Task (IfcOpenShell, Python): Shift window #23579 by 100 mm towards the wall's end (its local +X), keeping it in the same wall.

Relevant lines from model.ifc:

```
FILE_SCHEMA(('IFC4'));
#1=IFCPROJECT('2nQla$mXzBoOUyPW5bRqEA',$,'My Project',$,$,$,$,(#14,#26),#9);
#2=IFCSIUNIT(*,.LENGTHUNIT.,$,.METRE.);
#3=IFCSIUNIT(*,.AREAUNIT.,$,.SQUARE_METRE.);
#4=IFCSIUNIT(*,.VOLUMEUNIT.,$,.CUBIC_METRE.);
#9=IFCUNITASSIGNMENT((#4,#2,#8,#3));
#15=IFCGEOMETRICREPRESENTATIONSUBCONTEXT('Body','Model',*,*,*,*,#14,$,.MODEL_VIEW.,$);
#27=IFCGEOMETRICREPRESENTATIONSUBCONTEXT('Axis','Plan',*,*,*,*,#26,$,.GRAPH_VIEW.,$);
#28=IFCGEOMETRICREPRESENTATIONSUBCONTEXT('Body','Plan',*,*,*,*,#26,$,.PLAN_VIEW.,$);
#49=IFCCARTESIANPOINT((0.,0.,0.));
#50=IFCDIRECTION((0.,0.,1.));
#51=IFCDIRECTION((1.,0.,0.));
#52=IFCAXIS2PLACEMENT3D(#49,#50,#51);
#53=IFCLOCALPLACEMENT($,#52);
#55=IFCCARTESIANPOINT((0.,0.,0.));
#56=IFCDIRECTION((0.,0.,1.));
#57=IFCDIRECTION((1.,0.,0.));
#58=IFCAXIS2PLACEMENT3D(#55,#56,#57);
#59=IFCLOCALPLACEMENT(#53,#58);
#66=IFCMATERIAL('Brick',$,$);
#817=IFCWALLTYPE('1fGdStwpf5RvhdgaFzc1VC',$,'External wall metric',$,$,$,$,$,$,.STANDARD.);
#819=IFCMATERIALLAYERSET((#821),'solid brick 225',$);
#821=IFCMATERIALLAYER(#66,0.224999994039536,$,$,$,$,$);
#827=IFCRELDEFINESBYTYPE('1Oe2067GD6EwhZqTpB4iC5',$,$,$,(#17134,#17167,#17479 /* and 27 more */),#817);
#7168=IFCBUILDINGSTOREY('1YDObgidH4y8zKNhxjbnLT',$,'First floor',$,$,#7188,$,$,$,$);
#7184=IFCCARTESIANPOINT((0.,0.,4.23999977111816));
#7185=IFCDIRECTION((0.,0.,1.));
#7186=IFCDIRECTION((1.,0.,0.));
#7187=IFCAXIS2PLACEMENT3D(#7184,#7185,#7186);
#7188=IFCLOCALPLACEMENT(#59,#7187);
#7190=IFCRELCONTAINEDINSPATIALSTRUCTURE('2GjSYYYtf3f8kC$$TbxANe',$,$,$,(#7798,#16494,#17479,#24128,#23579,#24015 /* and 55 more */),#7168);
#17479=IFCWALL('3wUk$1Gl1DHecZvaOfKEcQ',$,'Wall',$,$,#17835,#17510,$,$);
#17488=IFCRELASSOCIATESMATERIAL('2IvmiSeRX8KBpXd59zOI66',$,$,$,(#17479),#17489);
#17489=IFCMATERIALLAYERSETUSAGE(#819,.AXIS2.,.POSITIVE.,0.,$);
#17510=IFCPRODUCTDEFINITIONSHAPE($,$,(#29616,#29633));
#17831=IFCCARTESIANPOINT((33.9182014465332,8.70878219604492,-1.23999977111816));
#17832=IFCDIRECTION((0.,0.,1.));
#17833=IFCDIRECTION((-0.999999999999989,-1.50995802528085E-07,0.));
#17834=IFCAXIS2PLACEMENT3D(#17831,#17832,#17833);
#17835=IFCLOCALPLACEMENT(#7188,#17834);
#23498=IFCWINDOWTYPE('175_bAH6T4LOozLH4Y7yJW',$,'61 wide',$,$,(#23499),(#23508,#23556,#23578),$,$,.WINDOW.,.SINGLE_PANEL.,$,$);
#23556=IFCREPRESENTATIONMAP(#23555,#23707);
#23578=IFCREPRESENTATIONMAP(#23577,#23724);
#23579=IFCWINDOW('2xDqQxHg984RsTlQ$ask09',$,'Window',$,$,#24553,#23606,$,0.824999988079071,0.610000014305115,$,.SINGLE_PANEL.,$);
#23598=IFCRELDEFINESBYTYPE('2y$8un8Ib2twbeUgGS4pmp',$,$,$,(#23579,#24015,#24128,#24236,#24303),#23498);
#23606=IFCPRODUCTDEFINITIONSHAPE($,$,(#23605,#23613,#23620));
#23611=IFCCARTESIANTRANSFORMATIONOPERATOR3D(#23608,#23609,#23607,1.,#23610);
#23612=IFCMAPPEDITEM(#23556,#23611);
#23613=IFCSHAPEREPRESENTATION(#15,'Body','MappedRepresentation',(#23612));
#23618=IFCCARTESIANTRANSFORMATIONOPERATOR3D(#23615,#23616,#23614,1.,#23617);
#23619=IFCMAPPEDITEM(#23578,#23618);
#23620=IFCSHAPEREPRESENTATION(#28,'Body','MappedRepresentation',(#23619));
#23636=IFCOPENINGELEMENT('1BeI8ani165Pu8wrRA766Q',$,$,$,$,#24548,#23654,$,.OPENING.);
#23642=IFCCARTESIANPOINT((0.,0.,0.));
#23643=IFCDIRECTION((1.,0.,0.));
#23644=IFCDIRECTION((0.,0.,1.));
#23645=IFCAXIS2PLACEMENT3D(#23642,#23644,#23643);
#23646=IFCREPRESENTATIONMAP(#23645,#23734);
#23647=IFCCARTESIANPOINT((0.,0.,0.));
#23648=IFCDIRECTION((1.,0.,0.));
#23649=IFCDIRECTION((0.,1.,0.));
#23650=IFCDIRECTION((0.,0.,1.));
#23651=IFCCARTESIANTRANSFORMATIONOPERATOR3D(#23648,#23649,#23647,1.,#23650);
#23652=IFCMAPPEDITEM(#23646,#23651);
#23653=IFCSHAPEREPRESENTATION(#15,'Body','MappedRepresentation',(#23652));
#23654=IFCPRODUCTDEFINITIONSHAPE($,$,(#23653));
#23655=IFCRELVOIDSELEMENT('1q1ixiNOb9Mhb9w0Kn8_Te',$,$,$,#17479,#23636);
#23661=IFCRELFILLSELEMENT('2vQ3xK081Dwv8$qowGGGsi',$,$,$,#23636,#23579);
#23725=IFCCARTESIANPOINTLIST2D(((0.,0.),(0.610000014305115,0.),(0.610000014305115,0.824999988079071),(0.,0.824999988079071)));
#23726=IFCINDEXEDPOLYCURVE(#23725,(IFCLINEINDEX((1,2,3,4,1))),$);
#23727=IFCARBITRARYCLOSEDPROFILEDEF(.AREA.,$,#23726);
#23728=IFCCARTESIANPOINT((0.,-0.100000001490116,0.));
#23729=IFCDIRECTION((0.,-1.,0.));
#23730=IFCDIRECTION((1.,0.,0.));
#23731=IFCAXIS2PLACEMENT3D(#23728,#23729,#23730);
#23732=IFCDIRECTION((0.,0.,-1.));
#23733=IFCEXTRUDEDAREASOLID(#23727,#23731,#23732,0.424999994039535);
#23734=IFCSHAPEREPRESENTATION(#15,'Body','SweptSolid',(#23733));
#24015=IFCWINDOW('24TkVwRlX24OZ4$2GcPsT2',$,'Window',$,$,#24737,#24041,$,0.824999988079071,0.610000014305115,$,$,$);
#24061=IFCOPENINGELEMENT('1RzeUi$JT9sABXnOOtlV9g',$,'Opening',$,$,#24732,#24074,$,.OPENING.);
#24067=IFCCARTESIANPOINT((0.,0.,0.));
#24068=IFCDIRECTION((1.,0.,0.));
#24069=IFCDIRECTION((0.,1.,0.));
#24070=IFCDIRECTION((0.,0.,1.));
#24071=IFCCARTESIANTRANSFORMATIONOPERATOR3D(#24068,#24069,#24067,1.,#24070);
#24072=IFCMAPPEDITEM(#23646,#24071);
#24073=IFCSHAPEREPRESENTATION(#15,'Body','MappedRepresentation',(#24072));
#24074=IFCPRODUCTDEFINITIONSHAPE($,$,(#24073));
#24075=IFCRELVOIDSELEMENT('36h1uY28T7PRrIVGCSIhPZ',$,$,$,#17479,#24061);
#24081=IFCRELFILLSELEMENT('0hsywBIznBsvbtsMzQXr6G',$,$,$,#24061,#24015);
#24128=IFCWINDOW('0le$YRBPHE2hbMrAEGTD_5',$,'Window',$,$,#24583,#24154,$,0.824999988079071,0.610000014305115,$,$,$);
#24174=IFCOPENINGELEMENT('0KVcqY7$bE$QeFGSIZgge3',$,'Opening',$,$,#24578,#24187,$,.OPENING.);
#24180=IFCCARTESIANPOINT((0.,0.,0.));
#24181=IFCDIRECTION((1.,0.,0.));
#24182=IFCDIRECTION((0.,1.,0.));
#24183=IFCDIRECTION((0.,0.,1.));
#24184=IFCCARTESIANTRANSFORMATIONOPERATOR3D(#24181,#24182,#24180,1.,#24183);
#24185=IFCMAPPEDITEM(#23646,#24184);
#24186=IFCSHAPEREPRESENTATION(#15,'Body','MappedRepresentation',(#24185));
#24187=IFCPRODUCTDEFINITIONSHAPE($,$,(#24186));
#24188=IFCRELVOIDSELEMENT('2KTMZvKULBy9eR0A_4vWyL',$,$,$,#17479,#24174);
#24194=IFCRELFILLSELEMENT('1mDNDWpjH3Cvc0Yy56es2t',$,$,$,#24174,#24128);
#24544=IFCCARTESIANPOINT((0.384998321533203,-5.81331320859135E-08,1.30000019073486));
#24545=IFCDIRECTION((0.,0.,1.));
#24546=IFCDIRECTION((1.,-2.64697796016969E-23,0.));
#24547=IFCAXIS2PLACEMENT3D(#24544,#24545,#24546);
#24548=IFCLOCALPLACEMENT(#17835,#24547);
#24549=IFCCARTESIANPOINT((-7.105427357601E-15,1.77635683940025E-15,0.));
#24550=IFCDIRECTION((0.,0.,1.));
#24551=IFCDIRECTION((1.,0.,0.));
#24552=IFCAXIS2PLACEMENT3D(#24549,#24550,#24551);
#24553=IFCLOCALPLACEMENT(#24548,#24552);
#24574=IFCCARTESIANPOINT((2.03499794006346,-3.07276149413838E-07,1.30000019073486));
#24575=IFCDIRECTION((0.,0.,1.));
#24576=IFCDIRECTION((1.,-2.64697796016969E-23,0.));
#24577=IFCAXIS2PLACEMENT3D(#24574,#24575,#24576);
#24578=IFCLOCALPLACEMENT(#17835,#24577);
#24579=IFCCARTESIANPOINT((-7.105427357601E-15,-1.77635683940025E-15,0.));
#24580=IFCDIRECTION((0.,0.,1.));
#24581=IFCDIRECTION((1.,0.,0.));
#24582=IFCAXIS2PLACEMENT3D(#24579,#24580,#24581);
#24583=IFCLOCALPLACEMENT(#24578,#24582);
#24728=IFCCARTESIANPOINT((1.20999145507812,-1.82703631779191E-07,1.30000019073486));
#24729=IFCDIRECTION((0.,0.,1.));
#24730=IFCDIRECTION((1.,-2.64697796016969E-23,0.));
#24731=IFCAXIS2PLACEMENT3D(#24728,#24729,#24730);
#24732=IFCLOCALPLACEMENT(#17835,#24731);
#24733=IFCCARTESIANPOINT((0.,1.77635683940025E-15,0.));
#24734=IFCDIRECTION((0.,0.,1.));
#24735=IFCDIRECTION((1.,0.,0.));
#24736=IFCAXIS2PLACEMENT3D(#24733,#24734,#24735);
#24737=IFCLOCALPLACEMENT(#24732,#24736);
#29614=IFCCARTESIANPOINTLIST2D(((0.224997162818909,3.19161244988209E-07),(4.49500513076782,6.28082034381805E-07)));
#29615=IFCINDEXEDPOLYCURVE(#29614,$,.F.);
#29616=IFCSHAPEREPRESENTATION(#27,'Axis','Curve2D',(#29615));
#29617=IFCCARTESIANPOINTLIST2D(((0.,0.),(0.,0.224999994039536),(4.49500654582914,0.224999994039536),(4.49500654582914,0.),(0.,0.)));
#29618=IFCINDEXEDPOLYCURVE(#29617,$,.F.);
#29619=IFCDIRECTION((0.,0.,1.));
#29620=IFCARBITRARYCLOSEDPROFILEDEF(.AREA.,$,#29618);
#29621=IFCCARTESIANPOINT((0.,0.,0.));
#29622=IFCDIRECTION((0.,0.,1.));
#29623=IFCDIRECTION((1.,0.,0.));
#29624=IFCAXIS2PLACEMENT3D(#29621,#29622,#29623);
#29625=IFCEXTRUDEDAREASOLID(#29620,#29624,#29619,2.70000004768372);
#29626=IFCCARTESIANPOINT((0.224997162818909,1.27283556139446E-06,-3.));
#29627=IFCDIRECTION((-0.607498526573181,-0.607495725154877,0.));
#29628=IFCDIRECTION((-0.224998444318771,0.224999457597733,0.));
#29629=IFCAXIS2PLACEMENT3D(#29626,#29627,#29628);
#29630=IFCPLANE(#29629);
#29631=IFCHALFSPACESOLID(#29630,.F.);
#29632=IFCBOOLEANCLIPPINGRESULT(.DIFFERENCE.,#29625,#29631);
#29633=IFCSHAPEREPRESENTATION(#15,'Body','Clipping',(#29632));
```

```python
import ifcopenshell
import ifcopenshell.api.geometry
import ifcopenshell.util.placement

model = ifcopenshell.open("model.ifc")

window = model.by_id(23579)
opening = window.FillsVoids[0].RelatingOpeningElement
wall = opening.VoidsElements[0].RelatingBuildingElement

wall_matrix = ifcopenshell.util.placement.get_local_placement(wall.ObjectPlacement)
shift = wall_matrix[:3, 0] * 0.1
before = ifcopenshell.util.placement.get_local_placement(window.ObjectPlacement)[:3, 3].copy()

# The window is placed relative to its opening, so it follows when the opening moves.
matrix = ifcopenshell.util.placement.get_local_placement(opening.ObjectPlacement)
matrix[:3, 3] += shift
ifcopenshell.api.geometry.edit_object_placement(
    model, product=opening, matrix=matrix, is_si=False, should_transform_children=True
)

after = ifcopenshell.util.placement.get_local_placement(window.ObjectPlacement)[:3, 3]
print("window moved by", (after - before).round(3) + 0.0)

model.write("model-out.ifc")
```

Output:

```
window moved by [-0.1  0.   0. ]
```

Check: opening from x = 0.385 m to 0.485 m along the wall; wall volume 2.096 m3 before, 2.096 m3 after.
